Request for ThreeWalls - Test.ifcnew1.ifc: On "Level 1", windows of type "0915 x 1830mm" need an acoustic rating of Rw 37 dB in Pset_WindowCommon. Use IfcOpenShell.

First a look at what the model holds.

```python
import ifcopenshell
import ifcopenshell.util.element

model = ifcopenshell.open("ThreeWalls - Test.ifcnew1.ifc")
print(model.schema)
storey = next(s for s in model.by_type("IfcBuildingStorey") if s.Name == "Level 1")
windows = [e for e in ifcopenshell.util.element.get_decomposition(storey) if e.is_a("IfcWindow")]
seen = {}
for e in windows:
    element_type = ifcopenshell.util.element.get_type(e)
    key = (element_type.Name if element_type != e and element_type else None, ifcopenshell.util.element.get_pset(e, "Pset_WindowCommon", "AcousticRating"))
    seen[key] = seen.get(key, 0) + 1
for (name, value), count in sorted(seen.items(), key=str):
    print(count, "x", name, "|", value)
```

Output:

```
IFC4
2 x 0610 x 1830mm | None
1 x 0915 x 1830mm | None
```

```python
import ifcopenshell
import ifcopenshell.api.pset
import ifcopenshell.util.element

model = ifcopenshell.open("ThreeWalls - Test.ifcnew1.ifc")

storey = next(s for s in model.by_type("IfcBuildingStorey") if s.Name == "Level 1")
windows = [e for e in ifcopenshell.util.element.get_decomposition(storey) if e.is_a("IfcWindow")]

count = 0
for e in windows:
    element_type = ifcopenshell.util.element.get_type(e)
    if element_type in (None, e) or element_type.Name != "0915 x 1830mm":
        continue
    # add_pset returns the element's existing set when there is one.
    pset = ifcopenshell.api.pset.add_pset(model, product=e, name="Pset_WindowCommon")
    ifcopenshell.api.pset.edit_pset(model, pset=pset, properties={"AcousticRating": "Rw 37 dB"})
    count += 1

print(count, "windows updated")

model.write("ThreeWalls - Test.ifcnew1_updated.ifc")
```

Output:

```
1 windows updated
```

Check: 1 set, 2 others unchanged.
